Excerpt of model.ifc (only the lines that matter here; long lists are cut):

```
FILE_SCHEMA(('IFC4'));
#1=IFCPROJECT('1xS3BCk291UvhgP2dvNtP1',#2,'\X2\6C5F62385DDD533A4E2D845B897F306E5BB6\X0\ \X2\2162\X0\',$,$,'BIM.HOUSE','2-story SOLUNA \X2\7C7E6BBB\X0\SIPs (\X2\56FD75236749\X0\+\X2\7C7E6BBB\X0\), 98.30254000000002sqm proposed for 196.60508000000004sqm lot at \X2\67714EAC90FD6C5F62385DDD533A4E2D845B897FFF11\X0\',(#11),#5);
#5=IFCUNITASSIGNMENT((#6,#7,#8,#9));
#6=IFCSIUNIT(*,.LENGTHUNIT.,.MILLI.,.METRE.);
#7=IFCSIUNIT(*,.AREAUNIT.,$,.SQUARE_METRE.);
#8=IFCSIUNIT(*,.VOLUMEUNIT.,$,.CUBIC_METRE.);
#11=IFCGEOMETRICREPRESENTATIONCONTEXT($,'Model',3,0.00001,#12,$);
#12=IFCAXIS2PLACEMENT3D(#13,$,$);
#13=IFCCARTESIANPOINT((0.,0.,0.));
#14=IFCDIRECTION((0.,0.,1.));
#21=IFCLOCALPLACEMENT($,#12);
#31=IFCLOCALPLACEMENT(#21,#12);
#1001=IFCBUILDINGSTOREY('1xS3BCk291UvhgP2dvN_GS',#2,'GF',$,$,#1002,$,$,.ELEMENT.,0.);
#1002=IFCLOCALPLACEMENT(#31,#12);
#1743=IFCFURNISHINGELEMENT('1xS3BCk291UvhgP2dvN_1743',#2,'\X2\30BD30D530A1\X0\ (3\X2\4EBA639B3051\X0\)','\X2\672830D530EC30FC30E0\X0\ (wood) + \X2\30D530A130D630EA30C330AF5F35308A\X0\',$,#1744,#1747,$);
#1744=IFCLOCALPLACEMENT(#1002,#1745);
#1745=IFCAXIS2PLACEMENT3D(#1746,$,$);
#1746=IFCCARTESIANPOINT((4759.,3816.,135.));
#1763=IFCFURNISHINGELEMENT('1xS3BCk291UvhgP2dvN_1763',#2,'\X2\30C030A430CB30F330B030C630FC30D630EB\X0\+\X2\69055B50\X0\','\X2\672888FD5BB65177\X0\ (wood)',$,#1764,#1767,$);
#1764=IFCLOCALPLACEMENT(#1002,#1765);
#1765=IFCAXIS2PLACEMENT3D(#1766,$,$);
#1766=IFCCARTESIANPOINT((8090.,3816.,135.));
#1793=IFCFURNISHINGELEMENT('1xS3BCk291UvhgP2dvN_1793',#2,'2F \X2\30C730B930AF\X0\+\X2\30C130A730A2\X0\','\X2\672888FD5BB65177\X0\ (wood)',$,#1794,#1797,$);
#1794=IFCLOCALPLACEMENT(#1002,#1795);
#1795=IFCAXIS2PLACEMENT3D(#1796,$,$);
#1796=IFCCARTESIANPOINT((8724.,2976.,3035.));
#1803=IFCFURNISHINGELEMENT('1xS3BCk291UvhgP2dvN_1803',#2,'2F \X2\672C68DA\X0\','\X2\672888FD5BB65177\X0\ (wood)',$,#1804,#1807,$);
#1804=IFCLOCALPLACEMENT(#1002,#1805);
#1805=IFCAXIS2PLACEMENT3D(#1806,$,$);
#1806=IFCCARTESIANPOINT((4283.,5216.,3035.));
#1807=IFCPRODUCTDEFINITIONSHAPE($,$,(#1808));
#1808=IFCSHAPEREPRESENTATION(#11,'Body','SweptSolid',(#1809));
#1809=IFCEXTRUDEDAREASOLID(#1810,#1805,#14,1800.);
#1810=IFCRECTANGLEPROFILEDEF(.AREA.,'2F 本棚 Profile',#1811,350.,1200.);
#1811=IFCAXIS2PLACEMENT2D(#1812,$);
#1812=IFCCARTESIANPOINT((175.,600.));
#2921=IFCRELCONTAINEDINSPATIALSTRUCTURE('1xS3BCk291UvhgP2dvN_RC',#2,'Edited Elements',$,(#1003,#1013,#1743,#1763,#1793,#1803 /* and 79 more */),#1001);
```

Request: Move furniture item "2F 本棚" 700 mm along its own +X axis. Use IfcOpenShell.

```python
import ifcopenshell
import ifcopenshell.api.geometry
import ifcopenshell.util.placement
import ifcopenshell.util.unit

model = ifcopenshell.open("model.ifc")
unit_scale = ifcopenshell.util.unit.calculate_unit_scale(model)

item = model.by_guid("1xS3BCk291UvhgP2dvN_1803")
matrix = ifcopenshell.util.placement.get_local_placement(item.ObjectPlacement)
matrix[:3, 3] += matrix[:3, 0] * 0.7 / unit_scale
ifcopenshell.api.geometry.edit_object_placement(model, product=item, matrix=matrix, is_si=False)

print(ifcopenshell.util.placement.get_local_placement(item.ObjectPlacement).round(3) + 0.0)

model.write("model_updated.ifc")
```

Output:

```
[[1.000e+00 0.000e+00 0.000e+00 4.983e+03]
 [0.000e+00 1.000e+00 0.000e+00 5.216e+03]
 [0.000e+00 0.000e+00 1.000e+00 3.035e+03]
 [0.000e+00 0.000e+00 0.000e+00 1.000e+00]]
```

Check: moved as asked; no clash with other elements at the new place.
